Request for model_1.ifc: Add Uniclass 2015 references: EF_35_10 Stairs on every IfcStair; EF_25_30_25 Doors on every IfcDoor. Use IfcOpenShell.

First a look at what the model holds.

```python
import ifcopenshell

model = ifcopenshell.open("model_1.ifc")
print(model.schema)
print("classifications:", [c.Name for c in model.by_type("IfcClassification")])
for ifc_class in ("IfcDoor", "IfcRoof", "IfcStair", "IfcWall", "IfcWindow"):
    print(ifc_class, len(model.by_type(ifc_class)))
```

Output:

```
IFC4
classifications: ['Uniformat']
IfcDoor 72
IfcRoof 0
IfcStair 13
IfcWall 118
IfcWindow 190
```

```python
import ifcopenshell
import ifcopenshell.api.classification

model = ifcopenshell.open("model_1.ifc")

system = ifcopenshell.api.classification.add_classification(model, classification="Uniclass 2015")

codes = {
    "IfcStair": ("EF_35_10", "Stairs"),
    "IfcDoor": ("EF_25_30_25", "Doors"),
}
for ifc_class, (code, name) in codes.items():
    products = model.by_type(ifc_class)
    ifcopenshell.api.classification.add_reference(
        model, products=products, classification=system, identification=code, name=name
    )
    print(code, len(products))

model.write("model_1_rev.ifc")
```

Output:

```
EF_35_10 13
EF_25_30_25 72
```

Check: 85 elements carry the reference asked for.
